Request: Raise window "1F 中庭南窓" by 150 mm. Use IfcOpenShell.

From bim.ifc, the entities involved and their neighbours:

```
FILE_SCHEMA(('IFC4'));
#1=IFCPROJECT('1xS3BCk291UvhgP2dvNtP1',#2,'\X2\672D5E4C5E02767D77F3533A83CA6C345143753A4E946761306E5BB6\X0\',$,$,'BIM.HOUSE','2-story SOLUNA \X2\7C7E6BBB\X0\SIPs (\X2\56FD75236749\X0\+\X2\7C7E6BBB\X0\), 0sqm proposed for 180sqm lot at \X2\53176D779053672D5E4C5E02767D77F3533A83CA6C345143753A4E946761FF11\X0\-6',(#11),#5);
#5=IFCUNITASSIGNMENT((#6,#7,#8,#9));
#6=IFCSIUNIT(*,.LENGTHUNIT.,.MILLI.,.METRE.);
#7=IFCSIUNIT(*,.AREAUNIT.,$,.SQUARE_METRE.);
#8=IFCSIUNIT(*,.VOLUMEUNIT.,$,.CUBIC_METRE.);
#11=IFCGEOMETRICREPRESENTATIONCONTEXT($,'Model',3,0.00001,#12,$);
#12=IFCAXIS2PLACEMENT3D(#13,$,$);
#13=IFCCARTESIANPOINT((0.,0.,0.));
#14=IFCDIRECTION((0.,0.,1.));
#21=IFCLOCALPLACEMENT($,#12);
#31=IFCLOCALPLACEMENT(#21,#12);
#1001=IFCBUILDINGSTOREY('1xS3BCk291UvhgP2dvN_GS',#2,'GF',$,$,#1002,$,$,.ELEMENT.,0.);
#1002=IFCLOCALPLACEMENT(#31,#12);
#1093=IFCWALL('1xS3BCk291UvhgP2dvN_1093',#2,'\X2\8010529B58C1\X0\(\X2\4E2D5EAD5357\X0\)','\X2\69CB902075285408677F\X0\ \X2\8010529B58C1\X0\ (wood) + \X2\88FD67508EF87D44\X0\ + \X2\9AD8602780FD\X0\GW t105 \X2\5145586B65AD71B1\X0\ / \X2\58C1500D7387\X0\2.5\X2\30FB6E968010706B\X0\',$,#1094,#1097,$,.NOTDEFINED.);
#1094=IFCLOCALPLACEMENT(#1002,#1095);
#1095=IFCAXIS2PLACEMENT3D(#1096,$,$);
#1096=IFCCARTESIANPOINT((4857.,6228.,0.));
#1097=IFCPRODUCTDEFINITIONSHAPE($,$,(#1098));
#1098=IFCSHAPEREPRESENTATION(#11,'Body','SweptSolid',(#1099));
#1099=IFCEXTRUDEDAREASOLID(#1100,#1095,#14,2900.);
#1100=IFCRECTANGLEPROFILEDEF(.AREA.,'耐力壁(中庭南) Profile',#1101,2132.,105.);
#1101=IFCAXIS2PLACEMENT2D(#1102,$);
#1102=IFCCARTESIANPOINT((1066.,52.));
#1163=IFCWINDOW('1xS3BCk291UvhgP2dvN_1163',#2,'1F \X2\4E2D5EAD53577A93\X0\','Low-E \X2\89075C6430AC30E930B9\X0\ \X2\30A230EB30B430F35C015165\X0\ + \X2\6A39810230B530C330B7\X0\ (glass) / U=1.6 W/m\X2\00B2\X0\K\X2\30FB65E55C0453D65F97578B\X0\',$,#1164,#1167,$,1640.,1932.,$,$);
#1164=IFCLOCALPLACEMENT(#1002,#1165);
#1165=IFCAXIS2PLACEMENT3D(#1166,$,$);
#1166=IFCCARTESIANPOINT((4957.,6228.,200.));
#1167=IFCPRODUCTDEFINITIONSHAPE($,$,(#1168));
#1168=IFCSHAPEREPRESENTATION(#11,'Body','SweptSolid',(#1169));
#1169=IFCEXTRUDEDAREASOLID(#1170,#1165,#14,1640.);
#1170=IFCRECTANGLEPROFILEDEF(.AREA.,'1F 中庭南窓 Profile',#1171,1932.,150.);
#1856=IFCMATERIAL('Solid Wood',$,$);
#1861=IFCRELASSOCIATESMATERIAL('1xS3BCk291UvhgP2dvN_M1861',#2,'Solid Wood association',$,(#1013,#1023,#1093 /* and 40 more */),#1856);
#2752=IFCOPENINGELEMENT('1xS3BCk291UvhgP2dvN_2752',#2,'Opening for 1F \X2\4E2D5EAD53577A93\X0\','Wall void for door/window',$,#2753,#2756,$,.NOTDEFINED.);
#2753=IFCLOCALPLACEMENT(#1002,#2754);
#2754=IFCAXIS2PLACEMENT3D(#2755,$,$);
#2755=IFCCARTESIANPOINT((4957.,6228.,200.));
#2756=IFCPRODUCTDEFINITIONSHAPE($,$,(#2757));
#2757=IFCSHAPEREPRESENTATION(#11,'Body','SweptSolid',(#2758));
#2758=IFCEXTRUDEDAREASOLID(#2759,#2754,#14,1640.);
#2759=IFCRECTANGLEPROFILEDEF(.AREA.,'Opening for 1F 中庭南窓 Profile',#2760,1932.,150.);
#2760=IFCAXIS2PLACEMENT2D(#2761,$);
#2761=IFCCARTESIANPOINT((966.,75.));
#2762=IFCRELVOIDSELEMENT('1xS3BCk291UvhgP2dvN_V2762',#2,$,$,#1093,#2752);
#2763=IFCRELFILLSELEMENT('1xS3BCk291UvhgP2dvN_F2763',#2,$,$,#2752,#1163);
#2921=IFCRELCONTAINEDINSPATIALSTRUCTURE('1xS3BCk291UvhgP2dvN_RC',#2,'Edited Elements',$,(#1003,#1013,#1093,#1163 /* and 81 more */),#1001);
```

```python
import numpy as np
import ifcopenshell
import ifcopenshell.api.geometry
import ifcopenshell.util.placement
import ifcopenshell.util.unit

model = ifcopenshell.open("bim.ifc")
unit_scale = ifcopenshell.util.unit.calculate_unit_scale(model)

window = model.by_guid("1xS3BCk291UvhgP2dvN_1163")
opening = window.FillsVoids[0].RelatingOpeningElement
dz = 0.15 / unit_scale

shift = np.array([0.0, 0.0, dz])
# The window is not placed relative to its opening, so move both.
for product in (opening, window):
    matrix = ifcopenshell.util.placement.get_local_placement(product.ObjectPlacement)
    matrix[:3, 3] += shift
    ifcopenshell.api.geometry.edit_object_placement(model, product=product, matrix=matrix, is_si=False)

print(f"moved by {dz * unit_scale:+.3f} m")

model.write("bim_v2.ifc")
```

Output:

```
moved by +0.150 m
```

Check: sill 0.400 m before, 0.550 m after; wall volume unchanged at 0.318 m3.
